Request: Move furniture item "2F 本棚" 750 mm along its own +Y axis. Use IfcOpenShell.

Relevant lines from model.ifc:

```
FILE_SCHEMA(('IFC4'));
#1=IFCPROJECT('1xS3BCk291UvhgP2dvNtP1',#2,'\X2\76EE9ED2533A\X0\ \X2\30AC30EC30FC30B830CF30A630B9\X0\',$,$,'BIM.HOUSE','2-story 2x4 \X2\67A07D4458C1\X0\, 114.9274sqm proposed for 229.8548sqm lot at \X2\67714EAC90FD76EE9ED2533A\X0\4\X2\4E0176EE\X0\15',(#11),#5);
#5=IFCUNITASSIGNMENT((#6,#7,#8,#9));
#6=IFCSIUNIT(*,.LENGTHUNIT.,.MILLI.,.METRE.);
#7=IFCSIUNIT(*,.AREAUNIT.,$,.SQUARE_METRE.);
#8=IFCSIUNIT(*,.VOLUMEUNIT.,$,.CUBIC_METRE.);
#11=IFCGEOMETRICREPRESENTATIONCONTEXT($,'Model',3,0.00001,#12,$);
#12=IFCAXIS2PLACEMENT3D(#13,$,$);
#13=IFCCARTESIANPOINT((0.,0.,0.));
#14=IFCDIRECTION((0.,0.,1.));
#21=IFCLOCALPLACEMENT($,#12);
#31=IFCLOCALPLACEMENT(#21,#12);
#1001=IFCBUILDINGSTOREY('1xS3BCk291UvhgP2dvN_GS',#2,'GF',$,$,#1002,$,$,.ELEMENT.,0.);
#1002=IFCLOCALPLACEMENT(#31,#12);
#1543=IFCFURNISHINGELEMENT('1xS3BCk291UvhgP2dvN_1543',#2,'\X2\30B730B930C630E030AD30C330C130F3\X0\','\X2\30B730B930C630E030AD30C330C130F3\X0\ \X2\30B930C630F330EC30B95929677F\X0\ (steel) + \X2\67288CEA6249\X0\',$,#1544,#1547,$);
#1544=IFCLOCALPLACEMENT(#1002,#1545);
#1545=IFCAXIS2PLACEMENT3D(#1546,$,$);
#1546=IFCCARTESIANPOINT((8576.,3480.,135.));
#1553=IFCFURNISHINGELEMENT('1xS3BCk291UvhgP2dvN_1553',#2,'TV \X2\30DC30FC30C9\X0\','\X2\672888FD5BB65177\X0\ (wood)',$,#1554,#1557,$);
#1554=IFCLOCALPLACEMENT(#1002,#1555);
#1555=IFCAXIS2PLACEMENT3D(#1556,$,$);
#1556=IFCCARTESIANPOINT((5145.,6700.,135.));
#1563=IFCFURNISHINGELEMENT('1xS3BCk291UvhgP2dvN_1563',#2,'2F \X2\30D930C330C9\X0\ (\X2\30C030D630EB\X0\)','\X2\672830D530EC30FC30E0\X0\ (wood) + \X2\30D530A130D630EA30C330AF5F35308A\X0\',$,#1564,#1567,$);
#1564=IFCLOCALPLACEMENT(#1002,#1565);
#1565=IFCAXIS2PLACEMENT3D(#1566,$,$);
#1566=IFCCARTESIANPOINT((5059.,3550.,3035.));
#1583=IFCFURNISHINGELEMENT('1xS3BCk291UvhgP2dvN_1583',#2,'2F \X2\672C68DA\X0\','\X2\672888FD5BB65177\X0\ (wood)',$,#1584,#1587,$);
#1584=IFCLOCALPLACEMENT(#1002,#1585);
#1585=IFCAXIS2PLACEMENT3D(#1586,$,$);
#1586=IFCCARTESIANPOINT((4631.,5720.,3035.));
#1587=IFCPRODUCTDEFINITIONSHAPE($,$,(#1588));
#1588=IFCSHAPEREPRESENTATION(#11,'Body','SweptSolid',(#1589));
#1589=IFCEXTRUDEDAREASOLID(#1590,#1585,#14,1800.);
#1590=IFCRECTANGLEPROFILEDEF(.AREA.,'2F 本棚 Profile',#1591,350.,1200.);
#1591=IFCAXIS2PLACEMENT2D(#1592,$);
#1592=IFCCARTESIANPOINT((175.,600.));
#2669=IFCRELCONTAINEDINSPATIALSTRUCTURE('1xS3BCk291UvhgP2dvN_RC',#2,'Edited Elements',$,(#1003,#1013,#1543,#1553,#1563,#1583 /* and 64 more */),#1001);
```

```python
import ifcopenshell
import ifcopenshell.api.geometry
import ifcopenshell.util.placement
import ifcopenshell.util.unit

model = ifcopenshell.open("model.ifc")
unit_scale = ifcopenshell.util.unit.calculate_unit_scale(model)

item = model.by_guid("1xS3BCk291UvhgP2dvN_1583")
matrix = ifcopenshell.util.placement.get_local_placement(item.ObjectPlacement)
matrix[:3, 3] += matrix[:3, 1] * 0.75 / unit_scale
ifcopenshell.api.geometry.edit_object_placement(model, product=item, matrix=matrix, is_si=False)

print(ifcopenshell.util.placement.get_local_placement(item.ObjectPlacement).round(3) + 0.0)

model.write("model_v2.ifc")
```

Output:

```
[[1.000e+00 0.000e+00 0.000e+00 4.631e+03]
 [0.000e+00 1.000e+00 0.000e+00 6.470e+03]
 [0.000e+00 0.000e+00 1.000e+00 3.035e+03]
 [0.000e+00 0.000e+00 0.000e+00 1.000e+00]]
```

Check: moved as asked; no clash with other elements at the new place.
